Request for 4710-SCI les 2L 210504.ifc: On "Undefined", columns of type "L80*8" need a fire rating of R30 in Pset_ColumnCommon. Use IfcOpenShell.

First a look at what the model holds.

```python
import ifcopenshell
import ifcopenshell.util.element

model = ifcopenshell.open("4710-SCI les 2L 210504.ifc")
print(model.schema)
storey = next(s for s in model.by_type("IfcBuildingStorey") if s.Name == "Undefined")
columns = [e for e in ifcopenshell.util.element.get_decomposition(storey) if e.is_a("IfcColumn")]
seen = {}
for e in columns:
    element_type = ifcopenshell.util.element.get_type(e)
    key = (element_type.Name if element_type != e and element_type else None, ifcopenshell.util.element.get_pset(e, "Pset_ColumnCommon", "FireRating"))
    seen[key] = seen.get(key, 0) + 1
for (name, value), count in sorted(seen.items(), key=str):
    print(count, "x", name, "|", value)
```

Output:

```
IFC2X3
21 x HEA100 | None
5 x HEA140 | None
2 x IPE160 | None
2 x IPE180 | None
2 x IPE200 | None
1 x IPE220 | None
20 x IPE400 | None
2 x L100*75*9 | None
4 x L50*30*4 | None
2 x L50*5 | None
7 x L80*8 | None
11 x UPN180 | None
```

```python
import ifcopenshell
import ifcopenshell.api.pset
import ifcopenshell.util.element

model = ifcopenshell.open("4710-SCI les 2L 210504.ifc")

storey = next(s for s in model.by_type("IfcBuildingStorey") if s.Name == "Undefined")
columns = [e for e in ifcopenshell.util.element.get_decomposition(storey) if e.is_a("IfcColumn")]

count = 0
for e in columns:
    element_type = ifcopenshell.util.element.get_type(e)
    if element_type in (None, e) or element_type.Name != "L80*8":
        continue
    found = ifcopenshell.util.element.get_pset(e, "Pset_ColumnCommon", should_inherit=False)
    if found:
        pset = model.by_id(found["id"])
        if len(ifcopenshell.util.element.get_elements_by_pset(pset)) > 1:
            pset = ifcopenshell.api.pset.unshare_pset(model, products=[e], pset=pset)[0]
    else:
        pset = ifcopenshell.api.pset.add_pset(model, product=e, name="Pset_ColumnCommon")
    ifcopenshell.api.pset.edit_pset(model, pset=pset, properties={"FireRating": "R30"})
    count += 1

print(count, "columns updated")

model.write("4710-SCI les 2L 210504_v2.ifc")
```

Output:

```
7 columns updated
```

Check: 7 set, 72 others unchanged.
